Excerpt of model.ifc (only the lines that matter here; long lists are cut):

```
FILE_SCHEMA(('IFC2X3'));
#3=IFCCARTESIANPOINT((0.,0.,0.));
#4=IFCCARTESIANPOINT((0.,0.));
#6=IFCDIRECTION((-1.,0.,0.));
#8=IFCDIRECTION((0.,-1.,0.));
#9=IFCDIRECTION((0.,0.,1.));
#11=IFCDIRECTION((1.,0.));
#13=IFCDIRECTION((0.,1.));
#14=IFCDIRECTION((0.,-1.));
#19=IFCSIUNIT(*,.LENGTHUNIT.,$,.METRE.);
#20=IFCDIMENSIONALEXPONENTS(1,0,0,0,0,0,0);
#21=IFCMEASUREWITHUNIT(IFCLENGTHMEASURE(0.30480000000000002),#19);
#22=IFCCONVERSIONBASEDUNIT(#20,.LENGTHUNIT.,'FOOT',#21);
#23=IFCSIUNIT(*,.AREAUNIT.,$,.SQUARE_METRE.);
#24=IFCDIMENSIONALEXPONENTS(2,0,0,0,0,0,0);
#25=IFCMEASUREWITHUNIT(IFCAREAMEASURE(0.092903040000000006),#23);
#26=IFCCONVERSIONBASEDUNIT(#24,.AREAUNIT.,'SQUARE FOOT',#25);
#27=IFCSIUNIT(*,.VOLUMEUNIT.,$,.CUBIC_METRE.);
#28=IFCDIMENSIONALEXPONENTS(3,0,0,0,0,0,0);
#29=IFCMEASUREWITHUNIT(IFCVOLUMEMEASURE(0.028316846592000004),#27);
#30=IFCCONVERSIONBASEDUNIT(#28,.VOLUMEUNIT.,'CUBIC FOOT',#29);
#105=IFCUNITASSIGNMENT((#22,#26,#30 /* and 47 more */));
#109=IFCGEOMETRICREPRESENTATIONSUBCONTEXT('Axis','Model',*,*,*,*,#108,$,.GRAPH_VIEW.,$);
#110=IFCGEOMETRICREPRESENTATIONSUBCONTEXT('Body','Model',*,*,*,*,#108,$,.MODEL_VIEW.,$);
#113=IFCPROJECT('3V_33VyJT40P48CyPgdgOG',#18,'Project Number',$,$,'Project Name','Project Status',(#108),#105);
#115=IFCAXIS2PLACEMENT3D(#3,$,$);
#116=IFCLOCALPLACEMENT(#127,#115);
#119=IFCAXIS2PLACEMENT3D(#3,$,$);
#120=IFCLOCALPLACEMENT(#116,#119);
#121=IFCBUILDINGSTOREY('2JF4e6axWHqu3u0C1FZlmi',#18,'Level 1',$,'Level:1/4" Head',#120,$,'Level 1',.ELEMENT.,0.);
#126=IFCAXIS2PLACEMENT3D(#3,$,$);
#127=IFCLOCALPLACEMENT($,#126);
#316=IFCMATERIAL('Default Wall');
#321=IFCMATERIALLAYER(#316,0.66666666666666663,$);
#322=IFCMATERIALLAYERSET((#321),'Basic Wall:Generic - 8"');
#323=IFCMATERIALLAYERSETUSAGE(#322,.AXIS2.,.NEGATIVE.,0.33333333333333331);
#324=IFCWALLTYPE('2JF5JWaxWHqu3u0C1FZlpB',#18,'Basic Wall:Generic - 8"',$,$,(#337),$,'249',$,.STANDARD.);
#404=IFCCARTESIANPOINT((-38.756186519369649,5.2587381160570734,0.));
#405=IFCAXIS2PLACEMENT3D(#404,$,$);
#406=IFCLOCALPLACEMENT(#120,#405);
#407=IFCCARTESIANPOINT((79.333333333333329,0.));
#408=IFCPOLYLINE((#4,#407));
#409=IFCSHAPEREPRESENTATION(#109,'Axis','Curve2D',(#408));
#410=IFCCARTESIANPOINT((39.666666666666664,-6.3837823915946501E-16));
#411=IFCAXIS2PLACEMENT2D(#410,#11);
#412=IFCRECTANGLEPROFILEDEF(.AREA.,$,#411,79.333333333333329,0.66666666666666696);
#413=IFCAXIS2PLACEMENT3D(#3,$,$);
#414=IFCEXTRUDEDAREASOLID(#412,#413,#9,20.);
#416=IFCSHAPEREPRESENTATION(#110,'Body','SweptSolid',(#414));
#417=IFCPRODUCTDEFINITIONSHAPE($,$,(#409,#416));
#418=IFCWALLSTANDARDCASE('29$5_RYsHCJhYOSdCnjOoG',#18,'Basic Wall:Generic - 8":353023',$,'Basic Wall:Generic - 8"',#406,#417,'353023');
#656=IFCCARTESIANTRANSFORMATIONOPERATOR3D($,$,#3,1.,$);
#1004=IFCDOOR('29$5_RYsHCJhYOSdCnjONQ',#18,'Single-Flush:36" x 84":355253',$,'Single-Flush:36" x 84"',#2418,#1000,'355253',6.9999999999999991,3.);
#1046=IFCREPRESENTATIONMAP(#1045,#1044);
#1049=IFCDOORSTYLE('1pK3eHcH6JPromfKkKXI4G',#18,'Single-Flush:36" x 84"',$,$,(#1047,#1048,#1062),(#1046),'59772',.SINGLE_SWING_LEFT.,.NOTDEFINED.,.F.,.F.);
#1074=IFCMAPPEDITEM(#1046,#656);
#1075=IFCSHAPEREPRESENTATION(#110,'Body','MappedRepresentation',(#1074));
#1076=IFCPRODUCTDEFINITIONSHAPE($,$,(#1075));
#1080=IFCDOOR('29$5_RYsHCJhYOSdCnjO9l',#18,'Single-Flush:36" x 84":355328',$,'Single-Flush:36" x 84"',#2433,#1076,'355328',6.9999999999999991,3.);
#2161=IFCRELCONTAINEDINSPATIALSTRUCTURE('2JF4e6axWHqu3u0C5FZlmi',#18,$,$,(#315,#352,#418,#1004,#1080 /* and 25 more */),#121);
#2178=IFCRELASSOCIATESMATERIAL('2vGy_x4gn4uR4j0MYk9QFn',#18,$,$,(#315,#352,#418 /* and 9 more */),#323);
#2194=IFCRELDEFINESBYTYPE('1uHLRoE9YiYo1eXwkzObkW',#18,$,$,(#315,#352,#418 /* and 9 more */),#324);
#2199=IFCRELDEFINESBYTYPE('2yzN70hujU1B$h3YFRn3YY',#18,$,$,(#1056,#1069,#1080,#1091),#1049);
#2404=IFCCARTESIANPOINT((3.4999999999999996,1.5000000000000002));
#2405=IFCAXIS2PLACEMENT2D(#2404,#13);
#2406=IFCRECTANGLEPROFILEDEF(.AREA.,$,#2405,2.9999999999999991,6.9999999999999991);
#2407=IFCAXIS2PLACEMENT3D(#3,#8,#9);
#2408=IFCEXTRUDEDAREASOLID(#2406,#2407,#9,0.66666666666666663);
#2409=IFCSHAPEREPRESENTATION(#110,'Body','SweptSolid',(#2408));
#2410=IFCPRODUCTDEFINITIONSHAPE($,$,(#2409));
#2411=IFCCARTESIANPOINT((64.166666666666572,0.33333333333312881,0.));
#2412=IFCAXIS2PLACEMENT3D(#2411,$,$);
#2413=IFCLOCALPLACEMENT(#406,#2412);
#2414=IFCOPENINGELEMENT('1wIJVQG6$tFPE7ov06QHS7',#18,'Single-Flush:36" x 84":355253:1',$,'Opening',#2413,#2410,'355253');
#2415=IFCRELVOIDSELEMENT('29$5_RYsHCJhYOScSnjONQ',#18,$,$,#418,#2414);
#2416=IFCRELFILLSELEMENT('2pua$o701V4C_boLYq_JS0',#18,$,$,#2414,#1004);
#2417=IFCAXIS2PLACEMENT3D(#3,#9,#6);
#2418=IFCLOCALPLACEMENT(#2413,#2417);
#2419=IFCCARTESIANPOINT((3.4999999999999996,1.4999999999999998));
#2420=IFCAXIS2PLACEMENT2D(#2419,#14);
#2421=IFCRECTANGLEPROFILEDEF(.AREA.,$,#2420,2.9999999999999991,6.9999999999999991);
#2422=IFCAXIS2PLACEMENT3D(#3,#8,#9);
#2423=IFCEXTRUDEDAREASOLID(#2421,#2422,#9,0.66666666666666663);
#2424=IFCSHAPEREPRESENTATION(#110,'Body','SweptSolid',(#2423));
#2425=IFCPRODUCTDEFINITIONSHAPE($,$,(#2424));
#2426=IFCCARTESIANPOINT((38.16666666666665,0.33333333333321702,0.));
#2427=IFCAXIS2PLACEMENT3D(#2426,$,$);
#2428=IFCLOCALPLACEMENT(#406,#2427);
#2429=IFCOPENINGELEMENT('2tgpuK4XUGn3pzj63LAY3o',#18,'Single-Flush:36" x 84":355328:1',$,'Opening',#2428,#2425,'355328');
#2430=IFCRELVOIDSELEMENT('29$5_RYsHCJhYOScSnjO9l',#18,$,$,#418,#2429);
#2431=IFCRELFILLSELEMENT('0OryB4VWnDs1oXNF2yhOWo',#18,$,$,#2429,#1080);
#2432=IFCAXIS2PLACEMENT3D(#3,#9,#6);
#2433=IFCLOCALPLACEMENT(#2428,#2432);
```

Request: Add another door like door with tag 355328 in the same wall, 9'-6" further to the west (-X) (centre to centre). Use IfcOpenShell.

```python
import ifcopenshell
import ifcopenshell.api.feature
import ifcopenshell.api.geometry
import ifcopenshell.api.root
import ifcopenshell.geom
import ifcopenshell.util.element
import ifcopenshell.util.placement
import ifcopenshell.util.shape
import ifcopenshell.util.unit

model = ifcopenshell.open("model.ifc")
unit_scale = ifcopenshell.util.unit.calculate_unit_scale(model)
settings = ifcopenshell.geom.settings()


def volume(element):
    """Net volume in cubic metres, openings subtracted."""
    shape = ifcopenshell.geom.create_shape(settings, element)
    return ifcopenshell.util.shape.get_volume(shape.geometry)


def reuse_history(source, copy):
    """copy_class also copies each property set's owner history, people and application; keep the originals."""
    for rel in copy.IsDefinedBy:
        if rel.is_a("IfcRelDefinesByProperties") and (history := rel.RelatingPropertyDefinition.OwnerHistory):
            rel.RelatingPropertyDefinition.OwnerHistory = source.OwnerHistory
            ifcopenshell.util.element.remove_deep2(model, history)


door = model.by_id(1080)
opening = door.FillsVoids[0].RelatingOpeningElement
wall = opening.VoidsElements[0].RelatingBuildingElement
before = volume(wall)
shift = ifcopenshell.util.placement.get_local_placement(wall.ObjectPlacement)[:3, 0] * -114 * 0.0254 / unit_scale

# copy_class copies the void relationship, type, container and properties, but no geometry.
new_opening = ifcopenshell.api.root.copy_class(model, product=opening)
new_opening.Representation = ifcopenshell.util.element.copy_deep(
    model, opening.Representation, exclude=["IfcGeometricRepresentationContext", "IfcRepresentationMap"]
)
new_opening.Name = 'Single-Flush:36" x 84"'
new_opening.Tag = None
new_door = ifcopenshell.api.root.copy_class(model, product=door)
new_door.Representation = ifcopenshell.util.element.copy_deep(
    model, door.Representation, exclude=["IfcGeometricRepresentationContext", "IfcRepresentationMap"]
)
new_door.Name = 'Single-Flush:36" x 84"'
new_door.Tag = None
reuse_history(door, new_door)
fills = ifcopenshell.api.feature.add_filling(model, opening=new_opening, element=new_door)
fills.OwnerHistory = new_door.OwnerHistory  # required in IFC2X3

for old, new in ((opening, new_opening), (door, new_door)):
    matrix = ifcopenshell.util.placement.get_local_placement(old.ObjectPlacement)
    matrix[:3, 3] += shift
    ifcopenshell.api.geometry.edit_object_placement(model, product=new, matrix=matrix, is_si=False)

after = volume(wall)

print(f"wall volume {before:.3f} -> {after:.3f} m3")

model.write("model-out.ifc")
```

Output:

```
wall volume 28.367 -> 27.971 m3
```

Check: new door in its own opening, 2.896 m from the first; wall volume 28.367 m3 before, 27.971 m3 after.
